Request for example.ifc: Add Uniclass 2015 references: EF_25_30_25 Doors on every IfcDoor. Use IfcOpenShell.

First a look at what the model holds.

```python
import ifcopenshell

model = ifcopenshell.open("example.ifc")
print(model.schema)
print("classifications:", [c.Name for c in model.by_type("IfcClassification")])
for ifc_class in ("IfcDoor", "IfcRoof", "IfcStair", "IfcWall", "IfcWindow"):
    print(ifc_class, len(model.by_type(ifc_class)))
```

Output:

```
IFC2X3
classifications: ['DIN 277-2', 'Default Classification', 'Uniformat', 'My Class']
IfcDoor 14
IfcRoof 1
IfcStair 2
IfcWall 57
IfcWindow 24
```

```python
import ifcopenshell
import ifcopenshell.api.classification

model = ifcopenshell.open("example.ifc")

# IFC2X3 requires Source and Edition and has no link from the project to the system.
system = model.create_entity("IfcClassification", Source="NBS", Edition="2015", Name="Uniclass 2015")

codes = {
    "IfcDoor": ("EF_25_30_25", "Doors"),
}
for ifc_class, (code, name) in codes.items():
    products = model.by_type(ifc_class)
    ifcopenshell.api.classification.add_reference(
        model, products=products, classification=system, identification=code, name=name
    )
    print(code, len(products))

model.write("example_updated.ifc")
```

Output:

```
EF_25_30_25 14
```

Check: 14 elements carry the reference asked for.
